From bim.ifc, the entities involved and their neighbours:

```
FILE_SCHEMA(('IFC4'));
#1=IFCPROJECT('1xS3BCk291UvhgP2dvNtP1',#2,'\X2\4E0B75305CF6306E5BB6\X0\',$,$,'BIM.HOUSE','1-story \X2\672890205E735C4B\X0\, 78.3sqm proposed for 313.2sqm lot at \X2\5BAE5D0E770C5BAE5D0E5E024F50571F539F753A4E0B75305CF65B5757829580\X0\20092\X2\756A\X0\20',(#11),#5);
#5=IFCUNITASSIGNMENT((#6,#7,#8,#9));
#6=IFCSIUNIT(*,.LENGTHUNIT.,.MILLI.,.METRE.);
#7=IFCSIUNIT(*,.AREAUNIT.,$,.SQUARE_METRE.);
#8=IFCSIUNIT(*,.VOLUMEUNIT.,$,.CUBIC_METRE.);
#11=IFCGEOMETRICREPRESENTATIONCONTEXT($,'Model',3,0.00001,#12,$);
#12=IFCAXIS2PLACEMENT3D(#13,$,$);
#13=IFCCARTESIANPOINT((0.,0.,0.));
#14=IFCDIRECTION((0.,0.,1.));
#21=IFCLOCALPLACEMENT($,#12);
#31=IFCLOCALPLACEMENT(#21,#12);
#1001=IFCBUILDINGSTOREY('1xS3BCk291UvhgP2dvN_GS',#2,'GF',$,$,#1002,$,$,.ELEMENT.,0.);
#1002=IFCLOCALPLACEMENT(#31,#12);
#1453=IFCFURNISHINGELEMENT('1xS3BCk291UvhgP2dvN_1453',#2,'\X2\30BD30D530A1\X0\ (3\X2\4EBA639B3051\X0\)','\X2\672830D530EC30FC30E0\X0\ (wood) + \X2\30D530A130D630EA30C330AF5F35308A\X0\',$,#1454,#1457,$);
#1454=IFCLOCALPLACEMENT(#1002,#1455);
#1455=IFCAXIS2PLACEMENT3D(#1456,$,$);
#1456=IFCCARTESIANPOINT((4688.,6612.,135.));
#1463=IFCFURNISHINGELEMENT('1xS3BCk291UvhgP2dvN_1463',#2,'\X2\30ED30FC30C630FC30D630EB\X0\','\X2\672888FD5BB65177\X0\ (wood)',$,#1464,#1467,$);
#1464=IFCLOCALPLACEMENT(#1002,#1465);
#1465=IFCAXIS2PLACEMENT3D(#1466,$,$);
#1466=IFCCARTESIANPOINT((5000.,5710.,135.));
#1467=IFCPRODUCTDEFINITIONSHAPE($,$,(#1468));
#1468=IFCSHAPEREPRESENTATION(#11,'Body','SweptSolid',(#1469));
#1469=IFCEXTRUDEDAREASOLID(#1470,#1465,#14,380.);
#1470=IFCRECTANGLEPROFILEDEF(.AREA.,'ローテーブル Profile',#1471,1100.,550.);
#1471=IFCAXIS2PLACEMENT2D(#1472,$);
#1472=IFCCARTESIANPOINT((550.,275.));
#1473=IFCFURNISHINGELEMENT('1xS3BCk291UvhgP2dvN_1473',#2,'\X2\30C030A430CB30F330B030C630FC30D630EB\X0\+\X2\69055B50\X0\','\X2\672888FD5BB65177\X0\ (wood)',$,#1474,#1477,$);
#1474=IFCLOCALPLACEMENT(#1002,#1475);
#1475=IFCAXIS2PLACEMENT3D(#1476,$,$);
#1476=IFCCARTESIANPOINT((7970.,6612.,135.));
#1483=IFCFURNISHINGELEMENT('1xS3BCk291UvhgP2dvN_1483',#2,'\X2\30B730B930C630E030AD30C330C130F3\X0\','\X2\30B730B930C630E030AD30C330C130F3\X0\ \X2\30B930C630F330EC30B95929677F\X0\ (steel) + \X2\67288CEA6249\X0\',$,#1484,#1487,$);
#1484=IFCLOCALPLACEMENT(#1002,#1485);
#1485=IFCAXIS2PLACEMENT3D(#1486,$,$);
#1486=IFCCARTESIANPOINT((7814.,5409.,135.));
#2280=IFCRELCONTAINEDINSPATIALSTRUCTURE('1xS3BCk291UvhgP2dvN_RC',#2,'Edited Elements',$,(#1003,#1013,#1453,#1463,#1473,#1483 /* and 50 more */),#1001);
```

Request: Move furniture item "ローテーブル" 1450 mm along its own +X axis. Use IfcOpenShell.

```python
import ifcopenshell
import ifcopenshell.api.geometry
import ifcopenshell.util.placement

model = ifcopenshell.open("bim.ifc")

item = model.by_guid("1xS3BCk291UvhgP2dvN_1463")
matrix = ifcopenshell.util.placement.get_local_placement(item.ObjectPlacement)
matrix[:3, 3] += matrix[:3, 0] * 1450.0
ifcopenshell.api.geometry.edit_object_placement(model, product=item, matrix=matrix, is_si=False)

print(ifcopenshell.util.placement.get_local_placement(item.ObjectPlacement).round(3) + 0.0)

model.write("bim_v2.ifc")
```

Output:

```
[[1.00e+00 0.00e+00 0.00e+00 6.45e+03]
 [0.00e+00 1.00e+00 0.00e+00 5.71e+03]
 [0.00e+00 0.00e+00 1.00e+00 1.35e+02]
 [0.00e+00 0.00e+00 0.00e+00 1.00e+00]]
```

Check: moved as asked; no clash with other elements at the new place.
